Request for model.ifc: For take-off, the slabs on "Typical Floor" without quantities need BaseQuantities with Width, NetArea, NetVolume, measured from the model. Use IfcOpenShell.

First a look at what the model holds.

```python
import ifcopenshell
import ifcopenshell.util.element
import ifcopenshell.util.unit

model = ifcopenshell.open("model.ifc")
print(model.schema)
for unit_type in ("LENGTHUNIT", "AREAUNIT", "VOLUMEUNIT"):
    print(unit_type, ifcopenshell.util.unit.calculate_unit_scale(model, unit_type))
storey = next(s for s in model.by_type("IfcBuildingStorey") if s.Name == "Typical Floor")
slabs = [e for e in ifcopenshell.util.element.get_decomposition(storey) if e.is_a("IfcSlab")]
for e in sorted(slabs, key=lambda e: e.id()):
    print(e.id(), e.is_a(), e.Name, list(ifcopenshell.util.element.get_psets(e, qtos_only=True)), sep=" | ")
```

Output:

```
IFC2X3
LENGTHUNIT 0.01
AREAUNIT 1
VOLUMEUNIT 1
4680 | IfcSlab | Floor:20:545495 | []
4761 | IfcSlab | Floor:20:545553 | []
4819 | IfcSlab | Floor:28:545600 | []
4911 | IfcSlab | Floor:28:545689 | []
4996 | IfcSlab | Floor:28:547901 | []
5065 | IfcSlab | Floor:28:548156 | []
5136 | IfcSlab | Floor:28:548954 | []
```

```python
import ifcopenshell
import ifcopenshell.api.pset
import ifcopenshell.geom
import ifcopenshell.util.element
import ifcopenshell.util.shape
import ifcopenshell.util.unit

model = ifcopenshell.open("model.ifc")
unit_scale = ifcopenshell.util.unit.calculate_unit_scale(model)
area_scale = ifcopenshell.util.unit.calculate_unit_scale(model, "AREAUNIT")
volume_scale = ifcopenshell.util.unit.calculate_unit_scale(model, "VOLUMEUNIT")
settings = ifcopenshell.geom.settings()

storey = next(s for s in model.by_type("IfcBuildingStorey") if s.Name == "Typical Floor")
slabs = [e for e in ifcopenshell.util.element.get_decomposition(storey) if e.is_a("IfcSlab")]

for e in sorted(slabs, key=lambda e: e.id()):
    if ifcopenshell.util.element.get_psets(e, qtos_only=True, should_inherit=False):
        continue
    # Geometry comes back in metres, in the element's own axes.
    shape = ifcopenshell.geom.create_shape(settings, e)
    values = {
        "Width": ifcopenshell.util.shape.get_z(shape.geometry) / unit_scale,
        "NetArea": ifcopenshell.util.shape.get_footprint_area(shape.geometry) / area_scale,
        "NetVolume": ifcopenshell.util.shape.get_volume(shape.geometry) / volume_scale,
    }
    qto = ifcopenshell.api.pset.add_qto(model, product=e, name="BaseQuantities")
    ifcopenshell.api.pset.edit_qto(model, qto=qto, properties=values)
    print(e.id(), {k: round(v, 3) for k, v in values.items()})

model.write("model_updated.ifc")
```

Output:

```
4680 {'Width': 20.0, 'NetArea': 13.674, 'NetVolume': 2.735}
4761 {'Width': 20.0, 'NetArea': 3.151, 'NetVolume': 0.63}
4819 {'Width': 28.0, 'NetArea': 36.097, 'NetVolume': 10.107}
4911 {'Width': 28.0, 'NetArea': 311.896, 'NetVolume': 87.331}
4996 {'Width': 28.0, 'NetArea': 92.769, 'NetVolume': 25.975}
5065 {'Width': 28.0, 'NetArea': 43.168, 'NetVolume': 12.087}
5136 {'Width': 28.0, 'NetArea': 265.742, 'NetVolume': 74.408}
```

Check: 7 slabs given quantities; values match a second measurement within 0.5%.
